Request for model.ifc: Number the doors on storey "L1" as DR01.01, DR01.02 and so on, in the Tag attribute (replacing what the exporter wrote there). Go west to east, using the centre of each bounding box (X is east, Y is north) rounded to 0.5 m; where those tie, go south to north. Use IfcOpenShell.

First a look at what the model holds.

```python
import ifcopenshell
import ifcopenshell.util.element
import ifcopenshell.util.placement

model = ifcopenshell.open("model.ifc")
print(model.schema)
storey = next(s for s in model.by_type("IfcBuildingStorey") if s.Name == "L1")
doors = [e for e in ifcopenshell.util.element.get_decomposition(storey) if e.is_a("IfcDoor")]
for e in sorted(doors, key=lambda e: e.id()):
    origin = ifcopenshell.util.placement.get_local_placement(e.ObjectPlacement)[:3, 3]
    print(e.id(), e.Tag, e.Name, origin.round(2) + 0.0, sep=" | ")
```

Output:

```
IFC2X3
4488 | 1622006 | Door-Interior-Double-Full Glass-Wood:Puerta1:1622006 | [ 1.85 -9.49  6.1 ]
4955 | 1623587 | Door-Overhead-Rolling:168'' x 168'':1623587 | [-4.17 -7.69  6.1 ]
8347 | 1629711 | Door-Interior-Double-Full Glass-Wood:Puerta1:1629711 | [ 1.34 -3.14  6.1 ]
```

```python
import ifcopenshell
import ifcopenshell.geom
import ifcopenshell.util.element
import ifcopenshell.util.shape

model = ifcopenshell.open("model.ifc")
settings = ifcopenshell.geom.settings()
settings.set("use-world-coords", True)


def centre(element):
    shape = ifcopenshell.geom.create_shape(settings, element)
    return ifcopenshell.util.shape.get_bbox_centroid(shape.geometry)


storey = next(s for s in model.by_type("IfcBuildingStorey") if s.Name == "L1")
doors = [e for e in ifcopenshell.util.element.get_decomposition(storey) if e.is_a("IfcDoor")]

# Insertion points can sit at a corner or the storey origin, so sort by the geometry (in metres).
centres = {e: centre(e) for e in doors}
doors.sort(key=lambda e: (round(centres[e][0] / 0.5), centres[e][1]))

for i, e in enumerate(doors, start=1):
    number = f"DR01.{i:02d}"
    e.Tag = number
    print(e.id(), number)

model.write("model_updated.ifc")
```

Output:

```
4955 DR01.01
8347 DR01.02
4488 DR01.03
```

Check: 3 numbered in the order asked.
